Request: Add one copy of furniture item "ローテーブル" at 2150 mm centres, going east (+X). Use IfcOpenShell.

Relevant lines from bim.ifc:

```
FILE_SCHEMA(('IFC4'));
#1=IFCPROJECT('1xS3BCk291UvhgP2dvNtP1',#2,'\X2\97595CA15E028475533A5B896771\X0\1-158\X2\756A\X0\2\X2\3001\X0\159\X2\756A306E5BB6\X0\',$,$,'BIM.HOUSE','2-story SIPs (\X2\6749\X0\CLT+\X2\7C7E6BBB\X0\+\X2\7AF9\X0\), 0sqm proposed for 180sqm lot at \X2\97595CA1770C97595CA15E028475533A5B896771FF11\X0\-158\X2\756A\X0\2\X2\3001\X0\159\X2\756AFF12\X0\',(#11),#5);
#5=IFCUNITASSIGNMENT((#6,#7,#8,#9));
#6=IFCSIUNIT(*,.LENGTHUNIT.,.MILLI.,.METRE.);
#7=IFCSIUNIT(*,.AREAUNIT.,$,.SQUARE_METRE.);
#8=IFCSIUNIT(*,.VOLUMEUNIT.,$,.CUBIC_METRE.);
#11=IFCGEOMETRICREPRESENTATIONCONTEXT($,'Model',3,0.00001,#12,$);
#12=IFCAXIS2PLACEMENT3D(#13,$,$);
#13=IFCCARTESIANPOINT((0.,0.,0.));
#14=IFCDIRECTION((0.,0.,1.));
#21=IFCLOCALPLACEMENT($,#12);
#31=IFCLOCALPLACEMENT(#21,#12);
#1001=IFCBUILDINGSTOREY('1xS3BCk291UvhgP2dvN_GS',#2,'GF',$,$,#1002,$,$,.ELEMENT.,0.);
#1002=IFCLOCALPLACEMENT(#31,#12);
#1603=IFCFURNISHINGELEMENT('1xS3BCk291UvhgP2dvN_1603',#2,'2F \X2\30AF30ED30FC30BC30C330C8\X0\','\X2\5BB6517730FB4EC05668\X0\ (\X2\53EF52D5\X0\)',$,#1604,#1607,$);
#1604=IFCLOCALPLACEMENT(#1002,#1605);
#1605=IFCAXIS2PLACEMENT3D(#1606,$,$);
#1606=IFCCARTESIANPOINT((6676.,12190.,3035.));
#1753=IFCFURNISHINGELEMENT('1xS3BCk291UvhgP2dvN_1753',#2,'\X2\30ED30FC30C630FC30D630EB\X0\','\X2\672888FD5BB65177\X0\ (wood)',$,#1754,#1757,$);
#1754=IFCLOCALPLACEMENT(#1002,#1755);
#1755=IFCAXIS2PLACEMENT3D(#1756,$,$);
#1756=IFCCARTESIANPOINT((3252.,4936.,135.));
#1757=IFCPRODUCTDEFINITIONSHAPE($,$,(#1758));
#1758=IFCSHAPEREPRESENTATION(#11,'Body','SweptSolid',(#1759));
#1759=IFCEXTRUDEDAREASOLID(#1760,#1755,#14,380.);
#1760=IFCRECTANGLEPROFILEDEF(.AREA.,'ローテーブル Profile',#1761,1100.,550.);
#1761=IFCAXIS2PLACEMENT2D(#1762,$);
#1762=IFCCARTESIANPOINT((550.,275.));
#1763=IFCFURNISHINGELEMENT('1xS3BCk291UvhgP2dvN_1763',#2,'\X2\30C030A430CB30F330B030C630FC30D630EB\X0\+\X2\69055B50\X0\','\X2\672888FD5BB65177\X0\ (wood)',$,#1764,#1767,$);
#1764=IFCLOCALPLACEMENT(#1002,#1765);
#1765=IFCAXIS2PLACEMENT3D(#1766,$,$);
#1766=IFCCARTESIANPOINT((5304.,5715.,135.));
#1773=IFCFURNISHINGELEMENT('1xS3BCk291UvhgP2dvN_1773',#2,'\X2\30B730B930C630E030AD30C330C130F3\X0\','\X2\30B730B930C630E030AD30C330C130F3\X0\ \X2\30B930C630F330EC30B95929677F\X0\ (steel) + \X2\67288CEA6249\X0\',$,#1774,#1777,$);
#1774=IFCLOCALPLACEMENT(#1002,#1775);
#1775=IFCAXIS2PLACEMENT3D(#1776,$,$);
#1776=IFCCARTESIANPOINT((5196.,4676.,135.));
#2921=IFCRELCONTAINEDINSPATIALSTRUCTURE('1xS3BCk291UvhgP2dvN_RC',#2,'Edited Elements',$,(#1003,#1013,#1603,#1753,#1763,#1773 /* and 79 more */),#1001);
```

```python
import numpy as np
import ifcopenshell
import ifcopenshell.api.geometry
import ifcopenshell.api.root
import ifcopenshell.util.element
import ifcopenshell.util.placement

model = ifcopenshell.open("bim.ifc")


def reuse_history(source, copy):
    """copy_class also copies each property set's owner history, people and application; keep the originals."""
    for rel in copy.IsDefinedBy:
        if rel.is_a("IfcRelDefinesByProperties") and (history := rel.RelatingPropertyDefinition.OwnerHistory):
            rel.RelatingPropertyDefinition.OwnerHistory = source.OwnerHistory
            ifcopenshell.util.element.remove_deep2(model, history)


source = model.by_guid("1xS3BCk291UvhgP2dvN_1753")
base = ifcopenshell.util.placement.get_local_placement(source.ObjectPlacement)
step = np.array([1.0, 0.0, 0.0]) * 2150.0

for i in range(1, 2):
    copy = ifcopenshell.api.root.copy_class(model, product=source)
    copy.Representation = ifcopenshell.util.element.copy_deep(
        model, source.Representation, exclude=["IfcGeometricRepresentationContext", "IfcRepresentationMap"]
    )
    reuse_history(source, copy)
    matrix = base.copy()
    matrix[:3, 3] += i * step
    print("added at", matrix[:3, 3].round(3) + 0.0)
    ifcopenshell.api.geometry.edit_object_placement(model, product=copy, matrix=matrix, is_si=False)

model.write("bim_edited.ifc")
```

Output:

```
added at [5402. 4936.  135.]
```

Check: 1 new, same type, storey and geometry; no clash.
